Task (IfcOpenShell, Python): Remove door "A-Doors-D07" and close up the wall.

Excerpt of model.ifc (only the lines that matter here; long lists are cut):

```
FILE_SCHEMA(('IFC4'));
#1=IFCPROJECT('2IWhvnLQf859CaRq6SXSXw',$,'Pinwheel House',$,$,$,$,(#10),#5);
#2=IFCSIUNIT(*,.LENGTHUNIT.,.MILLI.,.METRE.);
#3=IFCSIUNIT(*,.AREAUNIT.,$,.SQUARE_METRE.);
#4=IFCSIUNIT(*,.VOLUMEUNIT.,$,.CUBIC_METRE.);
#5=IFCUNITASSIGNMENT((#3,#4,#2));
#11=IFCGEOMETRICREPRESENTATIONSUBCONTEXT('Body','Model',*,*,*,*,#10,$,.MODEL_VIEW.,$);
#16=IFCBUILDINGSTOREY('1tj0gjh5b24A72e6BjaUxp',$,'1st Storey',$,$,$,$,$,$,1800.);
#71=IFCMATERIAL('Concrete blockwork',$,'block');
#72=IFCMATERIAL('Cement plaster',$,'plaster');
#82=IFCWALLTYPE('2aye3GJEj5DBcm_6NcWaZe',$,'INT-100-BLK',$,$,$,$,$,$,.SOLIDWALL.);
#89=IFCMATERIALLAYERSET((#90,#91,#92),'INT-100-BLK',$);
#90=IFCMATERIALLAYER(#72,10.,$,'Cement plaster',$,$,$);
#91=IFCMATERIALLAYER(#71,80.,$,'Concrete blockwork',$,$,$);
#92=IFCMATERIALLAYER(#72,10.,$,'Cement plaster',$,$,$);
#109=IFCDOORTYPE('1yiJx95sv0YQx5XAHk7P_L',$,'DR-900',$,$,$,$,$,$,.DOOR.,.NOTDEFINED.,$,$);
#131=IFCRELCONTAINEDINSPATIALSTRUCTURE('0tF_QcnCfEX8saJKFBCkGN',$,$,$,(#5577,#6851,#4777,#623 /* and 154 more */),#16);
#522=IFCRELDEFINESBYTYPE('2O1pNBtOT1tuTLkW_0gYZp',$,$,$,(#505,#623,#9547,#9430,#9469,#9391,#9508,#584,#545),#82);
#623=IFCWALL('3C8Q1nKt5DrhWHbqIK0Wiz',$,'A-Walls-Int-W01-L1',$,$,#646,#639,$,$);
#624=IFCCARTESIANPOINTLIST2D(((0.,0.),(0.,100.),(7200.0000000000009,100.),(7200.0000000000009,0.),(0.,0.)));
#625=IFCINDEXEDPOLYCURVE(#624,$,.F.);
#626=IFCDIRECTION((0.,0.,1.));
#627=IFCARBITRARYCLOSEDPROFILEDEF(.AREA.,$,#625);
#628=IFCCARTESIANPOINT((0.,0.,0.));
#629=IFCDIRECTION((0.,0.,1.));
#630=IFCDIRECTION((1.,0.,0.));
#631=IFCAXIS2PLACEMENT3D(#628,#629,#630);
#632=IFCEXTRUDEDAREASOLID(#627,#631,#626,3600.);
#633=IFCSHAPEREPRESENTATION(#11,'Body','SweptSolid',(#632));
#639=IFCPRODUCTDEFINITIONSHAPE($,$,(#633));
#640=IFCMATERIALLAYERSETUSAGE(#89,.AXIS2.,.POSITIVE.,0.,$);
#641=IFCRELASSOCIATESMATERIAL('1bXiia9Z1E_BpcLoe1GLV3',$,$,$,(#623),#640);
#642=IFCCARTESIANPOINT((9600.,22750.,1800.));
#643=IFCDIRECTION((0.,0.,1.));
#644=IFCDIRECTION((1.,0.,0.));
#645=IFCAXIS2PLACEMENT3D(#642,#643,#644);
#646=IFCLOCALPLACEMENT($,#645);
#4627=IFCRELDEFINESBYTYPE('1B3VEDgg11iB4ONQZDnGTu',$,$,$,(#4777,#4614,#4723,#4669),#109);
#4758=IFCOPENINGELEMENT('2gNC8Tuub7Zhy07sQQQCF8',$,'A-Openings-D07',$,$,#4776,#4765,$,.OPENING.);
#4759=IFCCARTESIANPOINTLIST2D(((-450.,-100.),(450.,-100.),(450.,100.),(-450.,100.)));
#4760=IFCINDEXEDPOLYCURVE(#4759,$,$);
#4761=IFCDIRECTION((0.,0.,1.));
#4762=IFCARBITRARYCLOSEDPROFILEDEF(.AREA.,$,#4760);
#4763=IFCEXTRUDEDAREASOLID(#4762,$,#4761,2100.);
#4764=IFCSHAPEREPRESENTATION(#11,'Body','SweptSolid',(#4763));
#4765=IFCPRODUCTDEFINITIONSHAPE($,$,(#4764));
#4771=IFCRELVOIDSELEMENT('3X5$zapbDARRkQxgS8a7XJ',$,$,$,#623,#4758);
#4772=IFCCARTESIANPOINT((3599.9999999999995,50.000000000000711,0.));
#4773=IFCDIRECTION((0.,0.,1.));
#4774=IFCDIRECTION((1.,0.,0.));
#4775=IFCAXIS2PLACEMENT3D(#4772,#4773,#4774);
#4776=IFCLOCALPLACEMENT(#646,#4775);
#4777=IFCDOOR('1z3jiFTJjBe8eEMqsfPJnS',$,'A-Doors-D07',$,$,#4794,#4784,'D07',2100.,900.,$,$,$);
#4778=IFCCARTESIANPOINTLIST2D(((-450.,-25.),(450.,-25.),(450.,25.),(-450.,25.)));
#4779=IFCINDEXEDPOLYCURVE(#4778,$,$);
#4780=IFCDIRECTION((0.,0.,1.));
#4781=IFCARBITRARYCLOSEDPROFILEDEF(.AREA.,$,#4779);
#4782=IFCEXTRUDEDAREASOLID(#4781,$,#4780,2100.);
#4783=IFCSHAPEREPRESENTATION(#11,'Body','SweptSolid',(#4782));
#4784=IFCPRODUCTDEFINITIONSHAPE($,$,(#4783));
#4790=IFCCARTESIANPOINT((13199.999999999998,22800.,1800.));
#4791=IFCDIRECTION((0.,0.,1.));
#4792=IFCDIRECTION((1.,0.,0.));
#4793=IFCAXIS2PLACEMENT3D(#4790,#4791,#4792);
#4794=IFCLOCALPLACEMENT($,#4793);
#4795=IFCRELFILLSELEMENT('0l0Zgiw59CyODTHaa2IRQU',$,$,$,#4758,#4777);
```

```python
import ifcopenshell
import ifcopenshell.api.feature
import ifcopenshell.api.root
import ifcopenshell.geom
import ifcopenshell.util.shape

model = ifcopenshell.open("model.ifc")
settings = ifcopenshell.geom.settings()


def volume(element):
    """Net volume in cubic metres, openings subtracted."""
    shape = ifcopenshell.geom.create_shape(settings, element)
    return ifcopenshell.util.shape.get_volume(shape.geometry)


door = model.by_id(4777)
opening = door.FillsVoids[0].RelatingOpeningElement
wall = opening.VoidsElements[0].RelatingBuildingElement
before = volume(wall)

ifcopenshell.api.root.remove_product(model, product=door)
ifcopenshell.api.feature.remove_feature(model, feature=opening)

after = volume(wall)

print(f"wall volume {before:.3f} -> {after:.3f} m3")

model.write("model_updated.ifc")
```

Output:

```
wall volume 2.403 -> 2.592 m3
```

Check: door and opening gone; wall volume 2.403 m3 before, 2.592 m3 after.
